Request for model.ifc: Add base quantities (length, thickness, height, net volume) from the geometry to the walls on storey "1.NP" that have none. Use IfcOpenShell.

First a look at what the model holds.

```python
import ifcopenshell
import ifcopenshell.util.element
import ifcopenshell.util.unit

model = ifcopenshell.open("model.ifc")
print(model.schema)
for unit_type in ("LENGTHUNIT", "AREAUNIT", "VOLUMEUNIT"):
    print(unit_type, ifcopenshell.util.unit.calculate_unit_scale(model, unit_type))
storey = next(s for s in model.by_type("IfcBuildingStorey") if s.Name == "1.NP")
walls = [e for e in ifcopenshell.util.element.get_decomposition(storey) if e.is_a("IfcWall")]
for e in sorted(walls, key=lambda e: e.id()):
    print(e.id(), e.is_a(), e.Name, list(ifcopenshell.util.element.get_psets(e, qtos_only=True)), sep=" | ")
```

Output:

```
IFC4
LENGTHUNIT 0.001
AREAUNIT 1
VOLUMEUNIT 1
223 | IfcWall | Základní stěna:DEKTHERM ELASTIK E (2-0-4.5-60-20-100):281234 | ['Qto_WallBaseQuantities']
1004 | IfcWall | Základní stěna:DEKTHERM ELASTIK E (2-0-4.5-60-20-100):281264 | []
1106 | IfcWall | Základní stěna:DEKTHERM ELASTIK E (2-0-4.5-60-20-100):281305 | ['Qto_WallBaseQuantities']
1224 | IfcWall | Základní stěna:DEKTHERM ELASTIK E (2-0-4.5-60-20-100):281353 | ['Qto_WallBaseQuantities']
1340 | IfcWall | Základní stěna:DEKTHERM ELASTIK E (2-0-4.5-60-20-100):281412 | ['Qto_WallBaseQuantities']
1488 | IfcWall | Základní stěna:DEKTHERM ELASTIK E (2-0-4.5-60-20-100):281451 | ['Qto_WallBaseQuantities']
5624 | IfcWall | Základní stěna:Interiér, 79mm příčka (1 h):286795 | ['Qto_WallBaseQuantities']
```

```python
import ifcopenshell
import ifcopenshell.api.pset
import ifcopenshell.geom
import ifcopenshell.util.element
import ifcopenshell.util.shape
import ifcopenshell.util.unit

model = ifcopenshell.open("model.ifc")
unit_scale = ifcopenshell.util.unit.calculate_unit_scale(model)
volume_scale = ifcopenshell.util.unit.calculate_unit_scale(model, "VOLUMEUNIT")
settings = ifcopenshell.geom.settings()

storey = next(s for s in model.by_type("IfcBuildingStorey") if s.Name == "1.NP")
walls = [e for e in ifcopenshell.util.element.get_decomposition(storey) if e.is_a("IfcWall")]

for e in sorted(walls, key=lambda e: e.id()):
    if ifcopenshell.util.element.get_psets(e, qtos_only=True, should_inherit=False):
        continue
    # Geometry comes back in metres, in the element's own axes.
    shape = ifcopenshell.geom.create_shape(settings, e)
    values = {
        "Length": ifcopenshell.util.shape.get_x(shape.geometry) / unit_scale,
        "Width": ifcopenshell.util.shape.get_y(shape.geometry) / unit_scale,
        "Height": ifcopenshell.util.shape.get_z(shape.geometry) / unit_scale,
        "NetVolume": ifcopenshell.util.shape.get_volume(shape.geometry) / volume_scale,
    }
    qto = ifcopenshell.api.pset.add_qto(model, product=e, name="Qto_WallBaseQuantities")
    ifcopenshell.api.pset.edit_qto(model, qto=qto, properties=values)
    print(e.id(), {k: round(v, 3) for k, v in values.items()})

model.write("model_v2.ifc")
```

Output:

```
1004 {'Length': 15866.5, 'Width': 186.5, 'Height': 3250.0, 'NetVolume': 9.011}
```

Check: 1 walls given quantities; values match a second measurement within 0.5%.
